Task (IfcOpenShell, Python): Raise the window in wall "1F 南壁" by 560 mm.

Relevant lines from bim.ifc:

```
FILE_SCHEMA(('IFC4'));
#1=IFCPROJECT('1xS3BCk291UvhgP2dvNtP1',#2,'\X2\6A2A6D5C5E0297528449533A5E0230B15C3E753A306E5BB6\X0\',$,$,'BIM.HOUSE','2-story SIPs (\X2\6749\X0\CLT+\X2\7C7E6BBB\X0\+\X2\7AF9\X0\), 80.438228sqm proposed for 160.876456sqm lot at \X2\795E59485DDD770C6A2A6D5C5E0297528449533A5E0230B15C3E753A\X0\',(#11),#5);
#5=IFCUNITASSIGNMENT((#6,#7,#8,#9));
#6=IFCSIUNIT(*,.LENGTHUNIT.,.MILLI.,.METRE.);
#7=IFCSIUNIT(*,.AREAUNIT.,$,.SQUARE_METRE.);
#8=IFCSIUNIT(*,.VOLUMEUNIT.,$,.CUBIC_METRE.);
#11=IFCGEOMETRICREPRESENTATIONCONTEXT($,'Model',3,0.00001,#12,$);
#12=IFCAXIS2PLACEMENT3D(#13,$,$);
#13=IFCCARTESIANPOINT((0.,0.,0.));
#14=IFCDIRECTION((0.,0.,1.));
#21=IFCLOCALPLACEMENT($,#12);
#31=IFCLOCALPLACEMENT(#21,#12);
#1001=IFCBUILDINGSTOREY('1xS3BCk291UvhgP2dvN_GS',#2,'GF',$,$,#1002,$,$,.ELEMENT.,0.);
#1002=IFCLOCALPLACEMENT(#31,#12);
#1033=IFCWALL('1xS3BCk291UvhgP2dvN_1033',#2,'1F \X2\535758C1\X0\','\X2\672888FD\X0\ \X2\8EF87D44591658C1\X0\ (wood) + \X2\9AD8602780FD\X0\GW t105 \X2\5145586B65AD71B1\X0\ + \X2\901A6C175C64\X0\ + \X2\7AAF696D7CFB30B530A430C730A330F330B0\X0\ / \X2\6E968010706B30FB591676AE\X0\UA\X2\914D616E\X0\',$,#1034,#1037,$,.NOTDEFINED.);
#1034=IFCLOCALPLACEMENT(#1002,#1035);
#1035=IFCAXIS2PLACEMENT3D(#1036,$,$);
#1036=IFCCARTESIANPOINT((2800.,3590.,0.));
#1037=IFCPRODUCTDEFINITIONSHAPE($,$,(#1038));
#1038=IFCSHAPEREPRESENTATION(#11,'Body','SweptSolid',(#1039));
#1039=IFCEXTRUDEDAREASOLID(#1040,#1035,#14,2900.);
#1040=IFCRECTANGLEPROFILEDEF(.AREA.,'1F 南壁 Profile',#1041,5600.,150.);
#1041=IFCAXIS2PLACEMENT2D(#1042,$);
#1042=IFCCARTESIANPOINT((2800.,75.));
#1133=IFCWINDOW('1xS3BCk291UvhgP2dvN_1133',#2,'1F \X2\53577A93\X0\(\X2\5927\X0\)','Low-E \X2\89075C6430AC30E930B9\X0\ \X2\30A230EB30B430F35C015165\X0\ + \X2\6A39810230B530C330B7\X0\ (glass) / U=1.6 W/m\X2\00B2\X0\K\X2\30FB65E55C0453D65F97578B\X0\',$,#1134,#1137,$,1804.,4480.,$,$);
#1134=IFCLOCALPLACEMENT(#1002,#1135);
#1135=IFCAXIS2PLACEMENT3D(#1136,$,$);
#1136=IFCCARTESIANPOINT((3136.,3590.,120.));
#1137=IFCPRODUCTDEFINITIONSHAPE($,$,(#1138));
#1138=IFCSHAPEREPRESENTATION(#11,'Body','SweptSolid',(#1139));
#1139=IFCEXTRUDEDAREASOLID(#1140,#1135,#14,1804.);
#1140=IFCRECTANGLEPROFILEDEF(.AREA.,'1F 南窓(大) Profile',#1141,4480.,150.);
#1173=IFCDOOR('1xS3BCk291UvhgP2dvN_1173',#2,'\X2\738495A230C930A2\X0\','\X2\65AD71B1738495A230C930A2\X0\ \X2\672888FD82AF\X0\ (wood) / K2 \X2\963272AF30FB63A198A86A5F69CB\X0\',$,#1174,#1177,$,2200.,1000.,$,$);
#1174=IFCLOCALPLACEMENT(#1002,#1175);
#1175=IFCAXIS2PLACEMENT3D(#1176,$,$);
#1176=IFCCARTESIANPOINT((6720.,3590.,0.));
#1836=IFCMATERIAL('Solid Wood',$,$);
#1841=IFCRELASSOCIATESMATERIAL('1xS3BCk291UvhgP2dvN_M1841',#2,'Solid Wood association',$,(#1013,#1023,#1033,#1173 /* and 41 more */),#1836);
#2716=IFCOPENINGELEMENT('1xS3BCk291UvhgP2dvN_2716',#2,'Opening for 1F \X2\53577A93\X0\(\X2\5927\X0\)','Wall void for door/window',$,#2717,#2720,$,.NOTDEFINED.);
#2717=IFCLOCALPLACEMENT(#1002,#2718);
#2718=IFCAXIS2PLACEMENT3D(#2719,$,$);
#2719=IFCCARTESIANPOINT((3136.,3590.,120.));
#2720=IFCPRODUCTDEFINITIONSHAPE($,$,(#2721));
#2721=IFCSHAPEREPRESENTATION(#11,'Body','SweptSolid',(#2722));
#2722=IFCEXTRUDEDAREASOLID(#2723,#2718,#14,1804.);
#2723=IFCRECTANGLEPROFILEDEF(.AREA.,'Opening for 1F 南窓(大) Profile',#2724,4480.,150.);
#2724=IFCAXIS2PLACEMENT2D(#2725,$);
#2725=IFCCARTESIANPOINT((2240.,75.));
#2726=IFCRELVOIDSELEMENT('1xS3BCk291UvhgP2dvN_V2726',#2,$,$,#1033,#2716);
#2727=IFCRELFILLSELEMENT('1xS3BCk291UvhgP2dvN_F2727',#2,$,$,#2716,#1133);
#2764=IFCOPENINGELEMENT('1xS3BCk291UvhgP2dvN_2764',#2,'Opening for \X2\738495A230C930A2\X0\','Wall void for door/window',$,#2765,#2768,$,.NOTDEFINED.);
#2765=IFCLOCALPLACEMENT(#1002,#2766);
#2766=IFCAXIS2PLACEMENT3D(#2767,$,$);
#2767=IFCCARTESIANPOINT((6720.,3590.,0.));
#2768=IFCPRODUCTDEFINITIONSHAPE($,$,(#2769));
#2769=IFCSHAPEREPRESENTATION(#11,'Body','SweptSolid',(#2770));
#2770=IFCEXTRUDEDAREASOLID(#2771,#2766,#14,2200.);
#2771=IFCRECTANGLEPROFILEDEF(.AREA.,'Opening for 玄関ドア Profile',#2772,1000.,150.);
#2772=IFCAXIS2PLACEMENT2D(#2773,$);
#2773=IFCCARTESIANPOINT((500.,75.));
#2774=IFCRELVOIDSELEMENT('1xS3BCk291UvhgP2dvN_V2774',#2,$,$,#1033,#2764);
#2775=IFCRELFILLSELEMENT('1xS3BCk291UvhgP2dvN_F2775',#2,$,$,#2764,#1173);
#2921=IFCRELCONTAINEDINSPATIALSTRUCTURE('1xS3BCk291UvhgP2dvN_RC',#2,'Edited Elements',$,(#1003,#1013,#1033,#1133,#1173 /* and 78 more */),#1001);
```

```python
import numpy as np
import ifcopenshell
import ifcopenshell.api.geometry
import ifcopenshell.util.placement
import ifcopenshell.util.unit

model = ifcopenshell.open("bim.ifc")
unit_scale = ifcopenshell.util.unit.calculate_unit_scale(model)

window = model.by_guid("1xS3BCk291UvhgP2dvN_1133")
opening = window.FillsVoids[0].RelatingOpeningElement
dz = 0.56 / unit_scale

shift = np.array([0.0, 0.0, dz])
# The window is not placed relative to its opening, so move both.
for product in (opening, window):
    matrix = ifcopenshell.util.placement.get_local_placement(product.ObjectPlacement)
    matrix[:3, 3] += shift
    ifcopenshell.api.geometry.edit_object_placement(model, product=product, matrix=matrix, is_si=False)

print(f"moved by {dz * unit_scale:+.3f} m")

model.write("bim_updated.ifc")
```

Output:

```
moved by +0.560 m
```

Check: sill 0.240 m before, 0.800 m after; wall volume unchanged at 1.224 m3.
